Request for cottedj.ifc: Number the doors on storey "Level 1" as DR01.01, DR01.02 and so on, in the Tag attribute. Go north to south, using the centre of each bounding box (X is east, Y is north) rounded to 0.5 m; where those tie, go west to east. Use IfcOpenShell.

First a look at what the model holds.

```python
import ifcopenshell
import ifcopenshell.util.element
import ifcopenshell.util.placement

model = ifcopenshell.open("cottedj.ifc")
print(model.schema)
storey = next(s for s in model.by_type("IfcBuildingStorey") if s.Name == "Level 1")
doors = [e for e in ifcopenshell.util.element.get_decomposition(storey) if e.is_a("IfcDoor")]
for e in sorted(doors, key=lambda e: e.id()):
    origin = ifcopenshell.util.placement.get_local_placement(e.ObjectPlacement)[:3, 3]
    print(e.id(), e.Tag, e.Name, origin.round(2) + 0.0, sep=" | ")
```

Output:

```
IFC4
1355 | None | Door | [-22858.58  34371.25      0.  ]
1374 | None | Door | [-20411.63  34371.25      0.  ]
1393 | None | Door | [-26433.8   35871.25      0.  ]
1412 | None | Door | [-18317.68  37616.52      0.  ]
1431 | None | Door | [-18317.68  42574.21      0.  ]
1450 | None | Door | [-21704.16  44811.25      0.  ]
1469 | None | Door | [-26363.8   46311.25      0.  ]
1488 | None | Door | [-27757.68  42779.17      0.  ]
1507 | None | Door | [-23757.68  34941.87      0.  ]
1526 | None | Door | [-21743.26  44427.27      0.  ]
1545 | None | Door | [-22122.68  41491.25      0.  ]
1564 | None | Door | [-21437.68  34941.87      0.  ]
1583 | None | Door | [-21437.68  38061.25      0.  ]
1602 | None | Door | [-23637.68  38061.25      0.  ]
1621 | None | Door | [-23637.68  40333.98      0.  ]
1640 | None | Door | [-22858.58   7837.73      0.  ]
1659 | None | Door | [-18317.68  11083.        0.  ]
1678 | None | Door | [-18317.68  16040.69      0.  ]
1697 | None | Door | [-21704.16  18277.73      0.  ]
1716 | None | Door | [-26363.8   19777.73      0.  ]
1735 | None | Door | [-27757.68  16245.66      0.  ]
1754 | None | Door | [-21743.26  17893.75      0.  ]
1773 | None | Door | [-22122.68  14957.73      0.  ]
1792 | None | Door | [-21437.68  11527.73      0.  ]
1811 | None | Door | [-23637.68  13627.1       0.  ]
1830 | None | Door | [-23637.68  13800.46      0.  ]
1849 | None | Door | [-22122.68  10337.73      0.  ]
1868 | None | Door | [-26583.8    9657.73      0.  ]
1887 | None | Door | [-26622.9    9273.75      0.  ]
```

```python
import ifcopenshell
import ifcopenshell.geom
import ifcopenshell.util.element
import ifcopenshell.util.shape

model = ifcopenshell.open("cottedj.ifc")
settings = ifcopenshell.geom.settings()
settings.set("use-world-coords", True)


def centre(element):
    shape = ifcopenshell.geom.create_shape(settings, element)
    return ifcopenshell.util.shape.get_bbox_centroid(shape.geometry)


storey = next(s for s in model.by_type("IfcBuildingStorey") if s.Name == "Level 1")
doors = [e for e in ifcopenshell.util.element.get_decomposition(storey) if e.is_a("IfcDoor")]

# Insertion points can sit at a corner or the storey origin, so sort by the geometry (in metres).
centres = {e: centre(e) for e in doors}
doors.sort(key=lambda e: (-round(centres[e][1] / 0.5), centres[e][0]))

for i, e in enumerate(doors, start=1):
    number = f"DR01.{i:02d}"
    e.Tag = number
    print(e.id(), number)

model.write("cottedj_updated.ifc")
```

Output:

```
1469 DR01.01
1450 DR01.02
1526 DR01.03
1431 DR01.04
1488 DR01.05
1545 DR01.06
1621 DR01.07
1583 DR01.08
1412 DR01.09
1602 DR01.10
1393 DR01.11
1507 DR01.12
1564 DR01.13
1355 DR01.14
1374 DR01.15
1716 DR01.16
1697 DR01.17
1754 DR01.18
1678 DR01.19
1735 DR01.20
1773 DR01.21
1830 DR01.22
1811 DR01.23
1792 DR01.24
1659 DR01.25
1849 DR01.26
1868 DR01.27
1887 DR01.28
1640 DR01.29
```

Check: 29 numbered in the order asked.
